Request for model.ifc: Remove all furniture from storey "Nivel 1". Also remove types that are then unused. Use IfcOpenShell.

First a look at what the model holds.

```python
import ifcopenshell
import ifcopenshell.util.element

model = ifcopenshell.open("model.ifc")
print(model.schema)
storey = next(s for s in model.by_type("IfcBuildingStorey") if s.Name == "Nivel 1")
furniture = [e for e in ifcopenshell.util.element.get_decomposition(storey) if e.is_a("IfcFurnishingElement")]
seen = {}
for e in furniture:
    element_type = ifcopenshell.util.element.get_type(e)
    name = element_type.Name if element_type not in (None, e) else None
    seen[name] = seen.get(name, 0) + 1
for name, count in sorted(seen.items(), key=str):
    print(count, "x", name)
```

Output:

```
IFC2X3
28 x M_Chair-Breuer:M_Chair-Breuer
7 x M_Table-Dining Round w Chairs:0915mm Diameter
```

```python
import ifcopenshell
import ifcopenshell.api.root
import ifcopenshell.util.element

model = ifcopenshell.open("model.ifc")

storey = next(s for s in model.by_type("IfcBuildingStorey") if s.Name == "Nivel 1")
furniture = [e for e in ifcopenshell.util.element.get_decomposition(storey) if e.is_a("IfcFurnishingElement")]
types = {ifcopenshell.util.element.get_type(e) for e in furniture} - {None, *furniture}

for e in furniture:
    ifcopenshell.api.root.remove_product(model, product=e)
print(len(furniture), "removed")

unused = [t for t in types if not ifcopenshell.util.element.get_types(t)]
for t in unused:
    ifcopenshell.api.root.remove_product(model, product=t)
print(len(unused), "unused types removed")

model.write("model_edited.ifc")
```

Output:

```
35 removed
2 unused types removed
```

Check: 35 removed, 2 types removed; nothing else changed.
